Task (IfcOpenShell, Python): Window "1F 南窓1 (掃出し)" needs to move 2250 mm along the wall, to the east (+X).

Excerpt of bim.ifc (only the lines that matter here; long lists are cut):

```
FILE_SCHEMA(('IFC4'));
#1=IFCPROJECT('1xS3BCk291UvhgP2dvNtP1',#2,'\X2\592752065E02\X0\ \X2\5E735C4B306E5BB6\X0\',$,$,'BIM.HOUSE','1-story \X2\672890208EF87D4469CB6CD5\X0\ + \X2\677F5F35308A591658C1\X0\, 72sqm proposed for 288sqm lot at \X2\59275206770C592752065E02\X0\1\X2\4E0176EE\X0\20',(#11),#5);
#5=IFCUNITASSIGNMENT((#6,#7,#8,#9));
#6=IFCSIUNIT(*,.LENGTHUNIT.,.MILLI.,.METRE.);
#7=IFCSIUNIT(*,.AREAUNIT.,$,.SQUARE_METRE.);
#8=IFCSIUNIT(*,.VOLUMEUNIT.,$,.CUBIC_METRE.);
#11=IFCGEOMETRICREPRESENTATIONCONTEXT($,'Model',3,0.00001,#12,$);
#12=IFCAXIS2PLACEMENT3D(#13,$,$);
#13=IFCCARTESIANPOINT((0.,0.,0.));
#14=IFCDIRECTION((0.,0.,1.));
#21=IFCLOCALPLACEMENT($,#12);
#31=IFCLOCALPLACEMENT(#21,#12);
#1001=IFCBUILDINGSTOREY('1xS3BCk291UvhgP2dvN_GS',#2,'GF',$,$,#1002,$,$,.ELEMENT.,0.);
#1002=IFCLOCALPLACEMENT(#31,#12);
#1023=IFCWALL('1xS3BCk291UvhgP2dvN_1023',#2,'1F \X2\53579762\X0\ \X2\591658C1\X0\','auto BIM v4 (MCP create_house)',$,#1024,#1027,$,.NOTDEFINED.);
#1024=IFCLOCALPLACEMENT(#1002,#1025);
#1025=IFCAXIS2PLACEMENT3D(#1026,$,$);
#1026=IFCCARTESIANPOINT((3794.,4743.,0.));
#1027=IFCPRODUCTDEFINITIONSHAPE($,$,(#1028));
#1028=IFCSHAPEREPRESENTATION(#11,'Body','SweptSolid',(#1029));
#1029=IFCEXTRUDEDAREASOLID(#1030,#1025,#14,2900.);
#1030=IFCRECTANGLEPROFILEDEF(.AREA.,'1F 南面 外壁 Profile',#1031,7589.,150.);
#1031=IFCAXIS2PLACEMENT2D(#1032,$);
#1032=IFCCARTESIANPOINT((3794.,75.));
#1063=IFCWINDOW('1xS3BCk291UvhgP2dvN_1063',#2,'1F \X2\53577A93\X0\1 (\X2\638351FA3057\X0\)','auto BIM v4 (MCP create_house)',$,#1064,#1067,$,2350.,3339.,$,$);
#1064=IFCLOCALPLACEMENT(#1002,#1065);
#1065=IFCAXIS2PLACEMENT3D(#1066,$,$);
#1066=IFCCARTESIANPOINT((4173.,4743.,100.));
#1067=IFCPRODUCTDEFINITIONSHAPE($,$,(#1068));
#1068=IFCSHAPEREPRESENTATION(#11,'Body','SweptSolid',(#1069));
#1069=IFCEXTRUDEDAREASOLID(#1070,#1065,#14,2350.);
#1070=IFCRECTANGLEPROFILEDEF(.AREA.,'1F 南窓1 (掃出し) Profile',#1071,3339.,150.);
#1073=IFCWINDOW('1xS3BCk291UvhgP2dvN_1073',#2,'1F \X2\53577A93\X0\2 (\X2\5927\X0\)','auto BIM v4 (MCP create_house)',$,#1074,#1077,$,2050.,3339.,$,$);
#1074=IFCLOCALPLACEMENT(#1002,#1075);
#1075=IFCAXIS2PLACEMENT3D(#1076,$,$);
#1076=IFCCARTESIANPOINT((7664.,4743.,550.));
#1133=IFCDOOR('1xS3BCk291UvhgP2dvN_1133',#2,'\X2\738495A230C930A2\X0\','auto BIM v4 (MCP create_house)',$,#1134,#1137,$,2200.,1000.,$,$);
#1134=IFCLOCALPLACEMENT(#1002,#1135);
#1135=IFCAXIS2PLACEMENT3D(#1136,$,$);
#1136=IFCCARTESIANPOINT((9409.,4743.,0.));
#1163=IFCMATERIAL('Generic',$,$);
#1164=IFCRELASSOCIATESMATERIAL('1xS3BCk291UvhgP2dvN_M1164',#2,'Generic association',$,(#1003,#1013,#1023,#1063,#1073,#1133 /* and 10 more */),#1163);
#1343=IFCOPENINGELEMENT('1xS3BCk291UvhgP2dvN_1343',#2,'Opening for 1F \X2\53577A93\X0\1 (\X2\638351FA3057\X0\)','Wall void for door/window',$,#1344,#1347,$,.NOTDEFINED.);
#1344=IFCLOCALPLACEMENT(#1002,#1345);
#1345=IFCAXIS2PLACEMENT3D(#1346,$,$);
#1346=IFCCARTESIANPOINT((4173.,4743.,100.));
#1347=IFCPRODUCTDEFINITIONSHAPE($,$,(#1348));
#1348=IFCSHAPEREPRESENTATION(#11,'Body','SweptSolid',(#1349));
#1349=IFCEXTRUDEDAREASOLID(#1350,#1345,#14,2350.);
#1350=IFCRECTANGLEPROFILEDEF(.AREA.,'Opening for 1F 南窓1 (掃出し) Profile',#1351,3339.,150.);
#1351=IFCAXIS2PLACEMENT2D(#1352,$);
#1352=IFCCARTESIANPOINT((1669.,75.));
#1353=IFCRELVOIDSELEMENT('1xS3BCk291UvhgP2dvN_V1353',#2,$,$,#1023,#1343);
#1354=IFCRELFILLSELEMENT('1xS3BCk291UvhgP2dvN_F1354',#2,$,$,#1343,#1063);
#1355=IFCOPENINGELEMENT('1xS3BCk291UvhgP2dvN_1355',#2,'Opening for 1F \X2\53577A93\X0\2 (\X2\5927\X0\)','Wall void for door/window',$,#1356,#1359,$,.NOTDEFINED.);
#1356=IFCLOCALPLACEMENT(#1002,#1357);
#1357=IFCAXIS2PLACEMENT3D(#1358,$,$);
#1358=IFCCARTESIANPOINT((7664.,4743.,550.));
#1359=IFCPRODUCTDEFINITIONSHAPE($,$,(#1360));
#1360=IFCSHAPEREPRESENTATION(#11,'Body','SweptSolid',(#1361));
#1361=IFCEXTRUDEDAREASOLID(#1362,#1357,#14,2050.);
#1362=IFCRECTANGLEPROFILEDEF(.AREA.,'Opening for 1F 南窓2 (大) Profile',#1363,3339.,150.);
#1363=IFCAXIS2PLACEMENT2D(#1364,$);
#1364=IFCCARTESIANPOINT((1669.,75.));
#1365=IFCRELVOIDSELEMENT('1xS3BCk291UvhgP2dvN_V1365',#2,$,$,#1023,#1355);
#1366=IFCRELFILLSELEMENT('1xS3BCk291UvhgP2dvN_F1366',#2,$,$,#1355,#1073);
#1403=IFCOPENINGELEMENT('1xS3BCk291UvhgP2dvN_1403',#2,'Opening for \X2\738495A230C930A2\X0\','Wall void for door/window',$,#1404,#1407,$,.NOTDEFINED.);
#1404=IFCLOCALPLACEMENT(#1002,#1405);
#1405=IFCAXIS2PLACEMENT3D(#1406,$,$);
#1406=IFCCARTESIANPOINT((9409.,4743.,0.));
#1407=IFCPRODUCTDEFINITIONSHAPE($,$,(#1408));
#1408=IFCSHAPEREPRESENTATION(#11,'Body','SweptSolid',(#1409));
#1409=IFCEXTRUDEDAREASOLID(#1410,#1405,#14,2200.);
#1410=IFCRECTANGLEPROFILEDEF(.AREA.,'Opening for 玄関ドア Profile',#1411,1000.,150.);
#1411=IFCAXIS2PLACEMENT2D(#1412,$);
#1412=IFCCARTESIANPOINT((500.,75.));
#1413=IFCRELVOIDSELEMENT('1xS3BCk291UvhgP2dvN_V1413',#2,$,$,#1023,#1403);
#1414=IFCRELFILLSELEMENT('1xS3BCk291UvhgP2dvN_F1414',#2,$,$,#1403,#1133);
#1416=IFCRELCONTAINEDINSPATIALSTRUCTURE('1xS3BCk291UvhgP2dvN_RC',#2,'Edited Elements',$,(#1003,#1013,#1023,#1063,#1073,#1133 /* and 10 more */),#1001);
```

```python
import ifcopenshell
import ifcopenshell.api.geometry
import ifcopenshell.util.placement
import ifcopenshell.util.unit

model = ifcopenshell.open("bim.ifc")
unit_scale = ifcopenshell.util.unit.calculate_unit_scale(model)

window = model.by_guid("1xS3BCk291UvhgP2dvN_1063")
opening = window.FillsVoids[0].RelatingOpeningElement
wall = opening.VoidsElements[0].RelatingBuildingElement

wall_matrix = ifcopenshell.util.placement.get_local_placement(wall.ObjectPlacement)
shift = wall_matrix[:3, 0] * 2.25 / unit_scale
before = ifcopenshell.util.placement.get_local_placement(window.ObjectPlacement)[:3, 3].copy()

# The window is not placed relative to its opening, so move both.
for product in (opening, window):
    matrix = ifcopenshell.util.placement.get_local_placement(product.ObjectPlacement)
    matrix[:3, 3] += shift
    ifcopenshell.api.geometry.edit_object_placement(model, product=product, matrix=matrix, is_si=False)

after = ifcopenshell.util.placement.get_local_placement(window.ObjectPlacement)[:3, 3]
print("window moved by", (after - before).round(3) + 0.0)

model.write("bim_edited.ifc")
```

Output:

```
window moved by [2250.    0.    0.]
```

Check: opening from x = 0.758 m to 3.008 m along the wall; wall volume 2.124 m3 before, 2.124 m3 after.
